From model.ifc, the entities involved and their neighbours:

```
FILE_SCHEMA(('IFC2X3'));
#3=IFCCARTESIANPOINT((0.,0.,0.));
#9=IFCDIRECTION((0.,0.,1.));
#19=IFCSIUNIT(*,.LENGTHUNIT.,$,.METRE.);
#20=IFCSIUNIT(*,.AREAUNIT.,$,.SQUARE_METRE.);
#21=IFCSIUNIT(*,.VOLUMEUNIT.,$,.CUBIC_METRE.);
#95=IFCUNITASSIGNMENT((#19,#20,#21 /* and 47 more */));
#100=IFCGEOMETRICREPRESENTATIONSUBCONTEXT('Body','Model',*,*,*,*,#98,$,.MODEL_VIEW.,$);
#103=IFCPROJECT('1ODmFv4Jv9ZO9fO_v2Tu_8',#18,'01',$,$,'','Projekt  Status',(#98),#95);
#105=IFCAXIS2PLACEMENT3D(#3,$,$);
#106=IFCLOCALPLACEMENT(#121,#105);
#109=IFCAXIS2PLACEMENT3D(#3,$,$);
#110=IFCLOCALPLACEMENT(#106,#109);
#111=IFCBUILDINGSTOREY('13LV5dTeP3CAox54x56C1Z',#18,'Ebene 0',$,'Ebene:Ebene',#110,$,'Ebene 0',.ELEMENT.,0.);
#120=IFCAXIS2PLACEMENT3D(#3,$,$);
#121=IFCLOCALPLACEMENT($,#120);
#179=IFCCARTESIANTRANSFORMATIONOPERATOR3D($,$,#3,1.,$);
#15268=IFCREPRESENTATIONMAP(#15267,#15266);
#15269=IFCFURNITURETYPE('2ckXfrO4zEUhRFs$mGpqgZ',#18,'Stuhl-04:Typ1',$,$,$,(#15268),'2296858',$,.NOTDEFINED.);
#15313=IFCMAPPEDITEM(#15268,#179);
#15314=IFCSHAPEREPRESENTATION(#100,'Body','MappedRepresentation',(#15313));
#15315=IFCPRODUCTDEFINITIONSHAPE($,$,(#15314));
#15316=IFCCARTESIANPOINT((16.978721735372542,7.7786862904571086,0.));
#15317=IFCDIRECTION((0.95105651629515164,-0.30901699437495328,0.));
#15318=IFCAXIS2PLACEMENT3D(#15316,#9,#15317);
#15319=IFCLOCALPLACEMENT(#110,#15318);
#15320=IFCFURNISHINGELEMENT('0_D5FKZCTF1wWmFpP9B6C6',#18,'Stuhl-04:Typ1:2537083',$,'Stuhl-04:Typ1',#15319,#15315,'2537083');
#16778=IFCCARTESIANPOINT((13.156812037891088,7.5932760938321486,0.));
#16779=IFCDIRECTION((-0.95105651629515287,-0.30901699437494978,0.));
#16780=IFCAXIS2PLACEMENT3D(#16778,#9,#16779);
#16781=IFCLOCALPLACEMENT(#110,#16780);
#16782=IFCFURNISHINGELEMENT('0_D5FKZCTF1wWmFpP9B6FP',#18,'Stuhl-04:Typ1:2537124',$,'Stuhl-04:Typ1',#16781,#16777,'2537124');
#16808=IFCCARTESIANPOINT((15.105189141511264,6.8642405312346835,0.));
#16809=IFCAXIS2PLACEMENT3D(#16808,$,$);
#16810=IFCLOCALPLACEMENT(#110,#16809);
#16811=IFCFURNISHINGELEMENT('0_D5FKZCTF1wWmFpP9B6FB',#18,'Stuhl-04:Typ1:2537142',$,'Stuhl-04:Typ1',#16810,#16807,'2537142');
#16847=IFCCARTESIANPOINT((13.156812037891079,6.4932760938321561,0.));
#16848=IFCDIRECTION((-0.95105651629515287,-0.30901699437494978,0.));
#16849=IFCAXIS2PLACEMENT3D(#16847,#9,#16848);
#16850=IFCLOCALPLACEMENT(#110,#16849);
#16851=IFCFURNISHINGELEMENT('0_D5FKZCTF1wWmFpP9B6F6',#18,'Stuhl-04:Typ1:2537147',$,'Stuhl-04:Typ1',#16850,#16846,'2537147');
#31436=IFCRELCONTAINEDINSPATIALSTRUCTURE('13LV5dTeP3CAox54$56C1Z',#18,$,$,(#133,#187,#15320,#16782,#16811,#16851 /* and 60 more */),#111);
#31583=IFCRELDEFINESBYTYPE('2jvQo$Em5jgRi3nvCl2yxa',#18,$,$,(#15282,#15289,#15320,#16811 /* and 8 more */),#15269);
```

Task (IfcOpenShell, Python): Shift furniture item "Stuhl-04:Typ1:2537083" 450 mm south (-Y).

```python
import ifcopenshell
import ifcopenshell.api.geometry
import ifcopenshell.util.placement

model = ifcopenshell.open("model.ifc")

item = model.by_guid("0_D5FKZCTF1wWmFpP9B6C6")
matrix = ifcopenshell.util.placement.get_local_placement(item.ObjectPlacement)
matrix[1, 3] -= 0.45
ifcopenshell.api.geometry.edit_object_placement(model, product=item, matrix=matrix, is_si=False)

print(ifcopenshell.util.placement.get_local_placement(item.ObjectPlacement).round(3) + 0.0)

model.write("model_updated.ifc")
```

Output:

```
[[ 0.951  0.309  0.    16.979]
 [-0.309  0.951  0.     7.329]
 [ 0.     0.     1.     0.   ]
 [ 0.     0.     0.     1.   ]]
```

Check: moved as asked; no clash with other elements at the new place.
